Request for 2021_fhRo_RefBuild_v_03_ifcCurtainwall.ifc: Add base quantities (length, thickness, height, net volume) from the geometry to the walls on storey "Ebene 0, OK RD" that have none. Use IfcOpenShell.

First a look at what the model holds.

```python
import ifcopenshell
import ifcopenshell.util.element
import ifcopenshell.util.unit

model = ifcopenshell.open("2021_fhRo_RefBuild_v_03_ifcCurtainwall.ifc")
print(model.schema)
for unit_type in ("LENGTHUNIT", "AREAUNIT", "VOLUMEUNIT"):
    print(unit_type, ifcopenshell.util.unit.calculate_unit_scale(model, unit_type))
storey = next(s for s in model.by_type("IfcBuildingStorey") if s.Name == "Ebene 0, OK RD")
walls = [e for e in ifcopenshell.util.element.get_decomposition(storey) if e.is_a("IfcWall")]
for e in sorted(walls, key=lambda e: e.id()):
    print(e.id(), e.is_a(), e.Name, list(ifcopenshell.util.element.get_psets(e, qtos_only=True)), sep=" | ")
```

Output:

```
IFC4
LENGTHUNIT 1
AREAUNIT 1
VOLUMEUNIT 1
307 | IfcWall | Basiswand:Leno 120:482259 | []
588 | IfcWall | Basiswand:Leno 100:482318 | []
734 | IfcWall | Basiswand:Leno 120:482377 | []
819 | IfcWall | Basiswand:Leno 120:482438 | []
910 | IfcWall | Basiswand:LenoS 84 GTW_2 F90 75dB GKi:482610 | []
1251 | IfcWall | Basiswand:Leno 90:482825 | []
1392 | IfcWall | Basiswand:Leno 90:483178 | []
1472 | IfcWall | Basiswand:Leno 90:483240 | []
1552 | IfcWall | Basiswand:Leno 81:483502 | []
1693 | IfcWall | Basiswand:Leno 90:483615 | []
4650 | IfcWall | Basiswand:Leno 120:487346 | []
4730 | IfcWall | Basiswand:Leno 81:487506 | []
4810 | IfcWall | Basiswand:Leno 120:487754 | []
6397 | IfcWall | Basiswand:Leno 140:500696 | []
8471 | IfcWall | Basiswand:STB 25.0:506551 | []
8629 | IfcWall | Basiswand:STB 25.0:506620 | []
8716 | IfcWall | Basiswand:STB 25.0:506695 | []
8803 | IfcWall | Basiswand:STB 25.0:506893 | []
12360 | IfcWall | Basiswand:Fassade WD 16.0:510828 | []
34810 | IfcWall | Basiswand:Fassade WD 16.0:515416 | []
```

```python
import ifcopenshell
import ifcopenshell.api.pset
import ifcopenshell.geom
import ifcopenshell.util.element
import ifcopenshell.util.shape
import ifcopenshell.util.unit

model = ifcopenshell.open("2021_fhRo_RefBuild_v_03_ifcCurtainwall.ifc")
unit_scale = ifcopenshell.util.unit.calculate_unit_scale(model)
volume_scale = ifcopenshell.util.unit.calculate_unit_scale(model, "VOLUMEUNIT")
settings = ifcopenshell.geom.settings()

storey = next(s for s in model.by_type("IfcBuildingStorey") if s.Name == "Ebene 0, OK RD")
walls = [e for e in ifcopenshell.util.element.get_decomposition(storey) if e.is_a("IfcWall")]

for e in sorted(walls, key=lambda e: e.id()):
    if ifcopenshell.util.element.get_psets(e, qtos_only=True, should_inherit=False):
        continue
    # Geometry comes back in metres, in the element's own axes.
    shape = ifcopenshell.geom.create_shape(settings, e)
    values = {
        "Length": ifcopenshell.util.shape.get_x(shape.geometry) / unit_scale,
        "Width": ifcopenshell.util.shape.get_y(shape.geometry) / unit_scale,
        "Height": ifcopenshell.util.shape.get_z(shape.geometry) / unit_scale,
        "NetVolume": ifcopenshell.util.shape.get_volume(shape.geometry) / volume_scale,
    }
    qto = ifcopenshell.api.pset.add_qto(model, product=e, name="Qto_WallBaseQuantities")
    ifcopenshell.api.pset.edit_qto(model, qto=qto, properties=values)
    print(e.id(), {k: round(v, 3) for k, v in values.items()})

model.write("2021_fhRo_RefBuild_v_03_ifcCurtainwall_edited.ifc")
```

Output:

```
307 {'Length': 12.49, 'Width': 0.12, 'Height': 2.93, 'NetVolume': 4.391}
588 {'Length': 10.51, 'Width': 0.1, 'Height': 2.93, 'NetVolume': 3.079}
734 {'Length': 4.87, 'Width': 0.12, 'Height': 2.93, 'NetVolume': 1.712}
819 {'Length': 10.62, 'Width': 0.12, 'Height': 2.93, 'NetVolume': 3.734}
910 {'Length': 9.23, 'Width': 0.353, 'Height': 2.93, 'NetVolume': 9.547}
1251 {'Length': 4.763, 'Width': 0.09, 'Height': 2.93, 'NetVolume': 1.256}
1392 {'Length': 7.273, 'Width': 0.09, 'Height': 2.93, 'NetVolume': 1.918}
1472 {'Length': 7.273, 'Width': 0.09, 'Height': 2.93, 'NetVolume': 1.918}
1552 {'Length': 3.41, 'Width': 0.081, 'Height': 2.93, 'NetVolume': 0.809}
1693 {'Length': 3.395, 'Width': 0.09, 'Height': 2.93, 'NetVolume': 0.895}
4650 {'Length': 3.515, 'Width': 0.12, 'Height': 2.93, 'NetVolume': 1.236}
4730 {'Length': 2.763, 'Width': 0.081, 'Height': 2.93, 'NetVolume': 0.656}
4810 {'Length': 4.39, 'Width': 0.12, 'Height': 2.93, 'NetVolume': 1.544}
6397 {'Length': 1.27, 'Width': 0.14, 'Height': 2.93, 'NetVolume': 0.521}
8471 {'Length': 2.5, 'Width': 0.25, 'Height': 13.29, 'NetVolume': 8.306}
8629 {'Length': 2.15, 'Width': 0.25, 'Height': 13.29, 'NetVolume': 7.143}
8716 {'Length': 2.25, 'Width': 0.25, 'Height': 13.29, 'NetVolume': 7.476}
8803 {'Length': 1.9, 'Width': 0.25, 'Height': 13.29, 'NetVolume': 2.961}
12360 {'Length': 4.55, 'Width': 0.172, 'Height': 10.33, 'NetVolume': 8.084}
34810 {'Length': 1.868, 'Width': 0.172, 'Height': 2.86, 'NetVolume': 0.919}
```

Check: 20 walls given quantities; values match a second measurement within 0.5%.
